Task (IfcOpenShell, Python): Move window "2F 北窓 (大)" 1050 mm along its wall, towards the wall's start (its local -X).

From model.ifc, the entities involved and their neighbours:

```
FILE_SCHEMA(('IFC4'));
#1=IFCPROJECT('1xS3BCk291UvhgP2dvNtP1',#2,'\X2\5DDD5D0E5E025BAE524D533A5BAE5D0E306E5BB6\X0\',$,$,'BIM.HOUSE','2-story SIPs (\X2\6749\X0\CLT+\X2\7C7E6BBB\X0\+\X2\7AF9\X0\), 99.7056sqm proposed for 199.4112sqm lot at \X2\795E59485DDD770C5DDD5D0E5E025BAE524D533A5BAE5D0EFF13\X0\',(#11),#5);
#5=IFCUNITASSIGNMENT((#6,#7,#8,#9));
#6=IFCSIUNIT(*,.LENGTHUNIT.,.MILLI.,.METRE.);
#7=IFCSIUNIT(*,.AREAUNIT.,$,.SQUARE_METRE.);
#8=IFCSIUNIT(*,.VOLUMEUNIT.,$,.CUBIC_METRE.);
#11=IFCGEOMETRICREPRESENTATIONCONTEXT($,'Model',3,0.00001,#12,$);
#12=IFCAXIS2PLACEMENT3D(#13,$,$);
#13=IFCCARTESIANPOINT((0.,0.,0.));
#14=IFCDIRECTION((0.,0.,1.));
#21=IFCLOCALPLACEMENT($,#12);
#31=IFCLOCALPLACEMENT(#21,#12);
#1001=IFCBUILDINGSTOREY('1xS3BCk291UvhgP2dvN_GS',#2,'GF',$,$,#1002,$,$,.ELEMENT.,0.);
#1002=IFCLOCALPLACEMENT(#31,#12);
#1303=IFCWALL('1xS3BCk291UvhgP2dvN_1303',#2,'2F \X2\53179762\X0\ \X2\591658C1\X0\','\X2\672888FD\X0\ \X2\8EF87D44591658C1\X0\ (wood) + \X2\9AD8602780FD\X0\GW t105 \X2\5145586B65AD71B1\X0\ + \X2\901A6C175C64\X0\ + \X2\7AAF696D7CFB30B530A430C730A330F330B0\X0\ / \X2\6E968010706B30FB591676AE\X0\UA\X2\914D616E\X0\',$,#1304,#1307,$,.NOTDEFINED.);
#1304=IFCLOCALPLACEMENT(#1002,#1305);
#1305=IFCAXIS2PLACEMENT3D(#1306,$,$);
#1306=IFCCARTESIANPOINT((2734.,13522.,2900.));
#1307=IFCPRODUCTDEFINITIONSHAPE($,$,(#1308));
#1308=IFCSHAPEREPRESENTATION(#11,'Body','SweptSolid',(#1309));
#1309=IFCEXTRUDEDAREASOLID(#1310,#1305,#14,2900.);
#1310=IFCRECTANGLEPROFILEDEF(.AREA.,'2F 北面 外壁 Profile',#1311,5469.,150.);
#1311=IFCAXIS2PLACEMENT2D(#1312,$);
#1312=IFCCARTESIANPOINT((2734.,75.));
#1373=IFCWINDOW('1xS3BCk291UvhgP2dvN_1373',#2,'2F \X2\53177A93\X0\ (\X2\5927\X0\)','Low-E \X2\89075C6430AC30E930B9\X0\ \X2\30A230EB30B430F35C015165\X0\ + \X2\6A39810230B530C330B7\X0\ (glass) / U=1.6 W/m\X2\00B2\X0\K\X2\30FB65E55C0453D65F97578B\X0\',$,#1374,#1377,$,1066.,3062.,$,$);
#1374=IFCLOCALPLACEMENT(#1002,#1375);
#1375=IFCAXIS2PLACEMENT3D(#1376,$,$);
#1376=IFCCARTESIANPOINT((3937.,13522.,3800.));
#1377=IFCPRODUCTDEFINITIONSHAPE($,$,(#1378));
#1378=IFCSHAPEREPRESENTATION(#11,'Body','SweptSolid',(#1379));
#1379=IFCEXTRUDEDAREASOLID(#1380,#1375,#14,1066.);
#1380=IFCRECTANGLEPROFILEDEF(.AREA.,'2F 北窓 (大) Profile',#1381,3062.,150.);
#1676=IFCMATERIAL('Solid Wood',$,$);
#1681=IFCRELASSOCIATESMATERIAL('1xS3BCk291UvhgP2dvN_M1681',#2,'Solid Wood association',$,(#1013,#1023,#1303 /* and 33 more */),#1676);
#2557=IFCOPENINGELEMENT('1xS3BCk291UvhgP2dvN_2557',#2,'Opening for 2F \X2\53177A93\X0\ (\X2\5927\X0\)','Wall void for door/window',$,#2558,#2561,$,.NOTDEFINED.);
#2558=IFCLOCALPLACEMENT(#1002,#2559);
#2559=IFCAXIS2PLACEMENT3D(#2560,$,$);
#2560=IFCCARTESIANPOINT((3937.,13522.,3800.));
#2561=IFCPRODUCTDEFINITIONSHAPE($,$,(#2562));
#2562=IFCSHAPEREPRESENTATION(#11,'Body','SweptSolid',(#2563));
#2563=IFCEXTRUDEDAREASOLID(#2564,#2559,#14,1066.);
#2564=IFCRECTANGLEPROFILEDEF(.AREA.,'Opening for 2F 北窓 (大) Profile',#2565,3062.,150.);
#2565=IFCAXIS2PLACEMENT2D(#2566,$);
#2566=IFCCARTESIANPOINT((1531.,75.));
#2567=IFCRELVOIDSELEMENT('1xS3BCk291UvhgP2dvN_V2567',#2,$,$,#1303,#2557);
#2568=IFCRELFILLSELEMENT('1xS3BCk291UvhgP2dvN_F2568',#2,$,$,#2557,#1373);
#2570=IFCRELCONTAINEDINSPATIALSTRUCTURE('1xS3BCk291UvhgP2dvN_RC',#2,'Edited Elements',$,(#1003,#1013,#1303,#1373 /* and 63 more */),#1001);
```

```python
import ifcopenshell
import ifcopenshell.api.geometry
import ifcopenshell.util.placement
import ifcopenshell.util.unit

model = ifcopenshell.open("model.ifc")
unit_scale = ifcopenshell.util.unit.calculate_unit_scale(model)

window = model.by_id(1373)
opening = window.FillsVoids[0].RelatingOpeningElement
wall = opening.VoidsElements[0].RelatingBuildingElement

wall_matrix = ifcopenshell.util.placement.get_local_placement(wall.ObjectPlacement)
shift = wall_matrix[:3, 0] * -1.05 / unit_scale
before = ifcopenshell.util.placement.get_local_placement(window.ObjectPlacement)[:3, 3].copy()

# The window is not placed relative to its opening, so move both.
for product in (opening, window):
    matrix = ifcopenshell.util.placement.get_local_placement(product.ObjectPlacement)
    matrix[:3, 3] += shift
    ifcopenshell.api.geometry.edit_object_placement(model, product=product, matrix=matrix, is_si=False)

after = ifcopenshell.util.placement.get_local_placement(window.ObjectPlacement)[:3, 3]
print("window moved by", (after - before).round(3) + 0.0)

model.write("model_v2.ifc")
```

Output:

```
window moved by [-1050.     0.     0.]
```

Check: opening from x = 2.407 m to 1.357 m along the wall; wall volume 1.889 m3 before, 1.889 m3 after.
